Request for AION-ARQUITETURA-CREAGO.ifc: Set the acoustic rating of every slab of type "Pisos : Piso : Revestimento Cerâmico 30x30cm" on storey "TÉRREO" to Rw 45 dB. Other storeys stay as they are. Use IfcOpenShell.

First a look at what the model holds.

```python
import ifcopenshell
import ifcopenshell.util.element

model = ifcopenshell.open("AION-ARQUITETURA-CREAGO.ifc")
print(model.schema)
storey = next(s for s in model.by_type("IfcBuildingStorey") if s.Name == "TÉRREO")
slabs = [e for e in ifcopenshell.util.element.get_decomposition(storey) if e.is_a("IfcSlab")]
seen = {}
for e in slabs:
    element_type = ifcopenshell.util.element.get_type(e)
    key = (element_type.Name if element_type != e and element_type else None, ifcopenshell.util.element.get_pset(e, "Pset_SlabCommon", "AcousticRating"))
    seen[key] = seen.get(key, 0) + 1
for (name, value), count in sorted(seen.items(), key=str):
    print(count, "x", name, "|", value)
```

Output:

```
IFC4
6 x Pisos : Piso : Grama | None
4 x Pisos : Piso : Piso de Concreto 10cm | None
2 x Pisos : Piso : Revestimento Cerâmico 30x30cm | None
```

```python
import ifcopenshell
import ifcopenshell.api.pset
import ifcopenshell.util.element

model = ifcopenshell.open("AION-ARQUITETURA-CREAGO.ifc")

storey = next(s for s in model.by_type("IfcBuildingStorey") if s.Name == "TÉRREO")
slabs = [e for e in ifcopenshell.util.element.get_decomposition(storey) if e.is_a("IfcSlab")]

count = 0
for e in slabs:
    element_type = ifcopenshell.util.element.get_type(e)
    if element_type in (None, e) or element_type.Name != "Pisos : Piso : Revestimento Cerâmico 30x30cm":
        continue
    # add_pset returns the element's existing set when there is one.
    pset = ifcopenshell.api.pset.add_pset(model, product=e, name="Pset_SlabCommon")
    ifcopenshell.api.pset.edit_pset(model, pset=pset, properties={"AcousticRating": "Rw 45 dB"})
    count += 1

print(count, "slabs updated")

model.write("AION-ARQUITETURA-CREAGO_updated.ifc")
```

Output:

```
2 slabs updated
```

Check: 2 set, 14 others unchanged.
